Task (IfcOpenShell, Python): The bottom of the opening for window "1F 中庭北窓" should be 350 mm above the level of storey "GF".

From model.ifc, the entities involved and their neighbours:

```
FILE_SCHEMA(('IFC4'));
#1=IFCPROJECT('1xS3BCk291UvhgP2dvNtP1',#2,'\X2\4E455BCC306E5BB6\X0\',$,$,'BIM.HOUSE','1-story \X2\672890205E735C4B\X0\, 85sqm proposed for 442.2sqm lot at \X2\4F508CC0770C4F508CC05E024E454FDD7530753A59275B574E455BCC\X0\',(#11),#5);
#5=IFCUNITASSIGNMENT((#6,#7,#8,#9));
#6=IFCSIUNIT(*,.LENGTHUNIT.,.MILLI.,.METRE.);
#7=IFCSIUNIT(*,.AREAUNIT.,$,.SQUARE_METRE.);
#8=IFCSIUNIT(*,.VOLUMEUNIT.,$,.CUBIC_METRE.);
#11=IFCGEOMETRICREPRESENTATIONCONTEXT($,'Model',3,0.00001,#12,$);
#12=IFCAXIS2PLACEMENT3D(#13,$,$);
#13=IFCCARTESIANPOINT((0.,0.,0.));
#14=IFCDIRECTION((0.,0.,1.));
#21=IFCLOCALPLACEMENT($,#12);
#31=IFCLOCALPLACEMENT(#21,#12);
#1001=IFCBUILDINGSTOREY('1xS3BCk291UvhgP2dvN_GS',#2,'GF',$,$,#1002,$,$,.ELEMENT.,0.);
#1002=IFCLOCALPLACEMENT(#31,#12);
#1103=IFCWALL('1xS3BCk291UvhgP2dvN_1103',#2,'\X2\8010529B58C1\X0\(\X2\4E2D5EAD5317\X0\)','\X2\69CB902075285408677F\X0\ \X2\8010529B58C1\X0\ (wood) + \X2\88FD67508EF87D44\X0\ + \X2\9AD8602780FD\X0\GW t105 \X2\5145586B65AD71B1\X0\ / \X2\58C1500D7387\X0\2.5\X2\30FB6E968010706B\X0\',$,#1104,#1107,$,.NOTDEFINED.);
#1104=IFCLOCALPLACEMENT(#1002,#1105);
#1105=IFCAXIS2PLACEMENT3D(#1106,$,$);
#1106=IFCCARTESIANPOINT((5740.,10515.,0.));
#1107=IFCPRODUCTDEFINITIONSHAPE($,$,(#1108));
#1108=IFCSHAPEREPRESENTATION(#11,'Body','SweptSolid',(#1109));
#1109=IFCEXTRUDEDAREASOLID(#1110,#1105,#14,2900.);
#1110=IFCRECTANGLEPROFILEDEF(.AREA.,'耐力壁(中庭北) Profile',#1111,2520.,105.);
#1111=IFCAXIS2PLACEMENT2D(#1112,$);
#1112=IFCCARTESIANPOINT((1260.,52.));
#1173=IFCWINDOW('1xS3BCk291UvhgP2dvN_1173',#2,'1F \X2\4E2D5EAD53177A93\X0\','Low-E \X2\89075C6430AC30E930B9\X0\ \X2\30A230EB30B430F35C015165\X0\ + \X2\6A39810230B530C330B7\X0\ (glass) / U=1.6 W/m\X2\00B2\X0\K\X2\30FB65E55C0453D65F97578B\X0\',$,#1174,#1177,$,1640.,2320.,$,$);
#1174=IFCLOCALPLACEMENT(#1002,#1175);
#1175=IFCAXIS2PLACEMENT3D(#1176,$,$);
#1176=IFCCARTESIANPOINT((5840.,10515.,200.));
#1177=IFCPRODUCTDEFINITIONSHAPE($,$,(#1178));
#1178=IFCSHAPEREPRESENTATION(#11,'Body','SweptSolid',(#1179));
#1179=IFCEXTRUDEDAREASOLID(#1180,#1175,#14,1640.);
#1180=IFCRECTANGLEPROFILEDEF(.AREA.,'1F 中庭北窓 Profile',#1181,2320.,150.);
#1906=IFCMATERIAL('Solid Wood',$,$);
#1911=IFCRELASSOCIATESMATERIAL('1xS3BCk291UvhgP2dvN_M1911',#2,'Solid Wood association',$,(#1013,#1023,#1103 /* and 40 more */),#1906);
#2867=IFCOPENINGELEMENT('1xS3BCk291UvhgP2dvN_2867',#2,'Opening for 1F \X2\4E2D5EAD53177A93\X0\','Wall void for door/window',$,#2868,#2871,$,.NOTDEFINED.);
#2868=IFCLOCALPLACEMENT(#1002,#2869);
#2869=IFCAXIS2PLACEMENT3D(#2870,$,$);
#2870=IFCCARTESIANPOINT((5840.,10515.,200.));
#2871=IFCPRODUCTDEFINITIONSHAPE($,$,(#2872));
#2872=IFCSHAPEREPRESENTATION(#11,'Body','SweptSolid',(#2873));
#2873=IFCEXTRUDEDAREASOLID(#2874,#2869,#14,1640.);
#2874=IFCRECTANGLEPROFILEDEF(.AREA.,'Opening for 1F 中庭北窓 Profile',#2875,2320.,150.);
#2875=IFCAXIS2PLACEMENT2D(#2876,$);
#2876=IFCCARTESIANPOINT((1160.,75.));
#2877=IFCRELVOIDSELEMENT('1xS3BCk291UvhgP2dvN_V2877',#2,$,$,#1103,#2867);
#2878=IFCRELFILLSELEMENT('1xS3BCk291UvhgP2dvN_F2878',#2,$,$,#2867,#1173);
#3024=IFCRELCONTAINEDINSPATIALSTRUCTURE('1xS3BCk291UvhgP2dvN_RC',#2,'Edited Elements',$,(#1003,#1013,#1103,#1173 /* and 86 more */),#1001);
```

```python
import numpy as np
import ifcopenshell
import ifcopenshell.api.geometry
import ifcopenshell.geom
import ifcopenshell.util.element
import ifcopenshell.util.placement
import ifcopenshell.util.shape
import ifcopenshell.util.unit

model = ifcopenshell.open("model.ifc")
unit_scale = ifcopenshell.util.unit.calculate_unit_scale(model)

window = model.by_guid("1xS3BCk291UvhgP2dvN_1173")
opening = window.FillsVoids[0].RelatingOpeningElement
storey = ifcopenshell.util.element.get_container(window, ifc_class="IfcBuildingStorey")
level = ifcopenshell.util.placement.get_local_placement(storey.ObjectPlacement)[2, 3]

# The opening's origin need not be at the sill, so measure its lowest point.
shape = ifcopenshell.geom.create_shape(ifcopenshell.geom.settings(), opening)
bottom = ifcopenshell.util.shape.get_shape_bottom_elevation(shape, shape.geometry) / unit_scale
dz = level + 0.35 / unit_scale - bottom

shift = np.array([0.0, 0.0, dz])
# The window is not placed relative to its opening, so move both.
for product in (opening, window):
    matrix = ifcopenshell.util.placement.get_local_placement(product.ObjectPlacement)
    matrix[:3, 3] += shift
    ifcopenshell.api.geometry.edit_object_placement(model, product=product, matrix=matrix, is_si=False)

print(f"moved by {dz * unit_scale:+.3f} m")

model.write("model_edited.ifc")
```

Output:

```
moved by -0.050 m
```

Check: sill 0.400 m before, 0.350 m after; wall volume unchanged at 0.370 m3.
